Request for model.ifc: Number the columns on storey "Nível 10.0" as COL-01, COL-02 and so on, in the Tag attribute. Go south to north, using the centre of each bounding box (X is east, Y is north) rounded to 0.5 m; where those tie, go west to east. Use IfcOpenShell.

First a look at what the model holds.

```python
import ifcopenshell
import ifcopenshell.util.element
import ifcopenshell.util.placement

model = ifcopenshell.open("model.ifc")
print(model.schema)
storey = next(s for s in model.by_type("IfcBuildingStorey") if s.Name == "Nível 10.0")
columns = [e for e in ifcopenshell.util.element.get_decomposition(storey) if e.is_a("IfcColumn")]
for e in sorted(columns, key=lambda e: e.id()):
    origin = ifcopenshell.util.placement.get_local_placement(e.ObjectPlacement)[:3, 3]
    print(e.id(), e.Tag, e.Name, origin.round(2) + 0.0, sep=" | ")
```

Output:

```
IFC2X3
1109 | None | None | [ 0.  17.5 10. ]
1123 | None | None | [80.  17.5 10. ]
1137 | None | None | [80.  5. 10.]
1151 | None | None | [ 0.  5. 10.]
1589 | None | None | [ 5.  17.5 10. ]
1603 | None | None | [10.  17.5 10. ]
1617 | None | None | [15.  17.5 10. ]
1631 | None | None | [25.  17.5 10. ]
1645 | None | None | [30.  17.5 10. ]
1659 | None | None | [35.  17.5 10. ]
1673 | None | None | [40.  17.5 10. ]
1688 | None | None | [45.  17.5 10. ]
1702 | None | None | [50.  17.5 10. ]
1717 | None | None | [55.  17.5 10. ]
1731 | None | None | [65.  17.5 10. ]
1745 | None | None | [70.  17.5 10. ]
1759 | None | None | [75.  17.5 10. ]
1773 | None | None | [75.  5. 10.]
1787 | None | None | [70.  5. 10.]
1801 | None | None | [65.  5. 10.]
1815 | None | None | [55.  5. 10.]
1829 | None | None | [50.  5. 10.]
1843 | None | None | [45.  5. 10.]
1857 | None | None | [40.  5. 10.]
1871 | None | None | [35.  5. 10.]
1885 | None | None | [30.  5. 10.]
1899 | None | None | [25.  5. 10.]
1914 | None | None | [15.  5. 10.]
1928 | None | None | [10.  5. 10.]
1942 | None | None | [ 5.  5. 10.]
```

```python
import ifcopenshell
import ifcopenshell.geom
import ifcopenshell.util.element
import ifcopenshell.util.shape

model = ifcopenshell.open("model.ifc")
settings = ifcopenshell.geom.settings()
settings.set("use-world-coords", True)


def centre(element):
    shape = ifcopenshell.geom.create_shape(settings, element)
    return ifcopenshell.util.shape.get_bbox_centroid(shape.geometry)


storey = next(s for s in model.by_type("IfcBuildingStorey") if s.Name == "Nível 10.0")
columns = [e for e in ifcopenshell.util.element.get_decomposition(storey) if e.is_a("IfcColumn")]

# Insertion points can sit at a corner or the storey origin, so sort by the geometry (in metres).
centres = {e: centre(e) for e in columns}
columns.sort(key=lambda e: (round(centres[e][1] / 0.5), centres[e][0]))

for i, e in enumerate(columns, start=1):
    number = f"COL-{i:02d}"
    e.Tag = number
    print(e.id(), number)

model.write("model_updated.ifc")
```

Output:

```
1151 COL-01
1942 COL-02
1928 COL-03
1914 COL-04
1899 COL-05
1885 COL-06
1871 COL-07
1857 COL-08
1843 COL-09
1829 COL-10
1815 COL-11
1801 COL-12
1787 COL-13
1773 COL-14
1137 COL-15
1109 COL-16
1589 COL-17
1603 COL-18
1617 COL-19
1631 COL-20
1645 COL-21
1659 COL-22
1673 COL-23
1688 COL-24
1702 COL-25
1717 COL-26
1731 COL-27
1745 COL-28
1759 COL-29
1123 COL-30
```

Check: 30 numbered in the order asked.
